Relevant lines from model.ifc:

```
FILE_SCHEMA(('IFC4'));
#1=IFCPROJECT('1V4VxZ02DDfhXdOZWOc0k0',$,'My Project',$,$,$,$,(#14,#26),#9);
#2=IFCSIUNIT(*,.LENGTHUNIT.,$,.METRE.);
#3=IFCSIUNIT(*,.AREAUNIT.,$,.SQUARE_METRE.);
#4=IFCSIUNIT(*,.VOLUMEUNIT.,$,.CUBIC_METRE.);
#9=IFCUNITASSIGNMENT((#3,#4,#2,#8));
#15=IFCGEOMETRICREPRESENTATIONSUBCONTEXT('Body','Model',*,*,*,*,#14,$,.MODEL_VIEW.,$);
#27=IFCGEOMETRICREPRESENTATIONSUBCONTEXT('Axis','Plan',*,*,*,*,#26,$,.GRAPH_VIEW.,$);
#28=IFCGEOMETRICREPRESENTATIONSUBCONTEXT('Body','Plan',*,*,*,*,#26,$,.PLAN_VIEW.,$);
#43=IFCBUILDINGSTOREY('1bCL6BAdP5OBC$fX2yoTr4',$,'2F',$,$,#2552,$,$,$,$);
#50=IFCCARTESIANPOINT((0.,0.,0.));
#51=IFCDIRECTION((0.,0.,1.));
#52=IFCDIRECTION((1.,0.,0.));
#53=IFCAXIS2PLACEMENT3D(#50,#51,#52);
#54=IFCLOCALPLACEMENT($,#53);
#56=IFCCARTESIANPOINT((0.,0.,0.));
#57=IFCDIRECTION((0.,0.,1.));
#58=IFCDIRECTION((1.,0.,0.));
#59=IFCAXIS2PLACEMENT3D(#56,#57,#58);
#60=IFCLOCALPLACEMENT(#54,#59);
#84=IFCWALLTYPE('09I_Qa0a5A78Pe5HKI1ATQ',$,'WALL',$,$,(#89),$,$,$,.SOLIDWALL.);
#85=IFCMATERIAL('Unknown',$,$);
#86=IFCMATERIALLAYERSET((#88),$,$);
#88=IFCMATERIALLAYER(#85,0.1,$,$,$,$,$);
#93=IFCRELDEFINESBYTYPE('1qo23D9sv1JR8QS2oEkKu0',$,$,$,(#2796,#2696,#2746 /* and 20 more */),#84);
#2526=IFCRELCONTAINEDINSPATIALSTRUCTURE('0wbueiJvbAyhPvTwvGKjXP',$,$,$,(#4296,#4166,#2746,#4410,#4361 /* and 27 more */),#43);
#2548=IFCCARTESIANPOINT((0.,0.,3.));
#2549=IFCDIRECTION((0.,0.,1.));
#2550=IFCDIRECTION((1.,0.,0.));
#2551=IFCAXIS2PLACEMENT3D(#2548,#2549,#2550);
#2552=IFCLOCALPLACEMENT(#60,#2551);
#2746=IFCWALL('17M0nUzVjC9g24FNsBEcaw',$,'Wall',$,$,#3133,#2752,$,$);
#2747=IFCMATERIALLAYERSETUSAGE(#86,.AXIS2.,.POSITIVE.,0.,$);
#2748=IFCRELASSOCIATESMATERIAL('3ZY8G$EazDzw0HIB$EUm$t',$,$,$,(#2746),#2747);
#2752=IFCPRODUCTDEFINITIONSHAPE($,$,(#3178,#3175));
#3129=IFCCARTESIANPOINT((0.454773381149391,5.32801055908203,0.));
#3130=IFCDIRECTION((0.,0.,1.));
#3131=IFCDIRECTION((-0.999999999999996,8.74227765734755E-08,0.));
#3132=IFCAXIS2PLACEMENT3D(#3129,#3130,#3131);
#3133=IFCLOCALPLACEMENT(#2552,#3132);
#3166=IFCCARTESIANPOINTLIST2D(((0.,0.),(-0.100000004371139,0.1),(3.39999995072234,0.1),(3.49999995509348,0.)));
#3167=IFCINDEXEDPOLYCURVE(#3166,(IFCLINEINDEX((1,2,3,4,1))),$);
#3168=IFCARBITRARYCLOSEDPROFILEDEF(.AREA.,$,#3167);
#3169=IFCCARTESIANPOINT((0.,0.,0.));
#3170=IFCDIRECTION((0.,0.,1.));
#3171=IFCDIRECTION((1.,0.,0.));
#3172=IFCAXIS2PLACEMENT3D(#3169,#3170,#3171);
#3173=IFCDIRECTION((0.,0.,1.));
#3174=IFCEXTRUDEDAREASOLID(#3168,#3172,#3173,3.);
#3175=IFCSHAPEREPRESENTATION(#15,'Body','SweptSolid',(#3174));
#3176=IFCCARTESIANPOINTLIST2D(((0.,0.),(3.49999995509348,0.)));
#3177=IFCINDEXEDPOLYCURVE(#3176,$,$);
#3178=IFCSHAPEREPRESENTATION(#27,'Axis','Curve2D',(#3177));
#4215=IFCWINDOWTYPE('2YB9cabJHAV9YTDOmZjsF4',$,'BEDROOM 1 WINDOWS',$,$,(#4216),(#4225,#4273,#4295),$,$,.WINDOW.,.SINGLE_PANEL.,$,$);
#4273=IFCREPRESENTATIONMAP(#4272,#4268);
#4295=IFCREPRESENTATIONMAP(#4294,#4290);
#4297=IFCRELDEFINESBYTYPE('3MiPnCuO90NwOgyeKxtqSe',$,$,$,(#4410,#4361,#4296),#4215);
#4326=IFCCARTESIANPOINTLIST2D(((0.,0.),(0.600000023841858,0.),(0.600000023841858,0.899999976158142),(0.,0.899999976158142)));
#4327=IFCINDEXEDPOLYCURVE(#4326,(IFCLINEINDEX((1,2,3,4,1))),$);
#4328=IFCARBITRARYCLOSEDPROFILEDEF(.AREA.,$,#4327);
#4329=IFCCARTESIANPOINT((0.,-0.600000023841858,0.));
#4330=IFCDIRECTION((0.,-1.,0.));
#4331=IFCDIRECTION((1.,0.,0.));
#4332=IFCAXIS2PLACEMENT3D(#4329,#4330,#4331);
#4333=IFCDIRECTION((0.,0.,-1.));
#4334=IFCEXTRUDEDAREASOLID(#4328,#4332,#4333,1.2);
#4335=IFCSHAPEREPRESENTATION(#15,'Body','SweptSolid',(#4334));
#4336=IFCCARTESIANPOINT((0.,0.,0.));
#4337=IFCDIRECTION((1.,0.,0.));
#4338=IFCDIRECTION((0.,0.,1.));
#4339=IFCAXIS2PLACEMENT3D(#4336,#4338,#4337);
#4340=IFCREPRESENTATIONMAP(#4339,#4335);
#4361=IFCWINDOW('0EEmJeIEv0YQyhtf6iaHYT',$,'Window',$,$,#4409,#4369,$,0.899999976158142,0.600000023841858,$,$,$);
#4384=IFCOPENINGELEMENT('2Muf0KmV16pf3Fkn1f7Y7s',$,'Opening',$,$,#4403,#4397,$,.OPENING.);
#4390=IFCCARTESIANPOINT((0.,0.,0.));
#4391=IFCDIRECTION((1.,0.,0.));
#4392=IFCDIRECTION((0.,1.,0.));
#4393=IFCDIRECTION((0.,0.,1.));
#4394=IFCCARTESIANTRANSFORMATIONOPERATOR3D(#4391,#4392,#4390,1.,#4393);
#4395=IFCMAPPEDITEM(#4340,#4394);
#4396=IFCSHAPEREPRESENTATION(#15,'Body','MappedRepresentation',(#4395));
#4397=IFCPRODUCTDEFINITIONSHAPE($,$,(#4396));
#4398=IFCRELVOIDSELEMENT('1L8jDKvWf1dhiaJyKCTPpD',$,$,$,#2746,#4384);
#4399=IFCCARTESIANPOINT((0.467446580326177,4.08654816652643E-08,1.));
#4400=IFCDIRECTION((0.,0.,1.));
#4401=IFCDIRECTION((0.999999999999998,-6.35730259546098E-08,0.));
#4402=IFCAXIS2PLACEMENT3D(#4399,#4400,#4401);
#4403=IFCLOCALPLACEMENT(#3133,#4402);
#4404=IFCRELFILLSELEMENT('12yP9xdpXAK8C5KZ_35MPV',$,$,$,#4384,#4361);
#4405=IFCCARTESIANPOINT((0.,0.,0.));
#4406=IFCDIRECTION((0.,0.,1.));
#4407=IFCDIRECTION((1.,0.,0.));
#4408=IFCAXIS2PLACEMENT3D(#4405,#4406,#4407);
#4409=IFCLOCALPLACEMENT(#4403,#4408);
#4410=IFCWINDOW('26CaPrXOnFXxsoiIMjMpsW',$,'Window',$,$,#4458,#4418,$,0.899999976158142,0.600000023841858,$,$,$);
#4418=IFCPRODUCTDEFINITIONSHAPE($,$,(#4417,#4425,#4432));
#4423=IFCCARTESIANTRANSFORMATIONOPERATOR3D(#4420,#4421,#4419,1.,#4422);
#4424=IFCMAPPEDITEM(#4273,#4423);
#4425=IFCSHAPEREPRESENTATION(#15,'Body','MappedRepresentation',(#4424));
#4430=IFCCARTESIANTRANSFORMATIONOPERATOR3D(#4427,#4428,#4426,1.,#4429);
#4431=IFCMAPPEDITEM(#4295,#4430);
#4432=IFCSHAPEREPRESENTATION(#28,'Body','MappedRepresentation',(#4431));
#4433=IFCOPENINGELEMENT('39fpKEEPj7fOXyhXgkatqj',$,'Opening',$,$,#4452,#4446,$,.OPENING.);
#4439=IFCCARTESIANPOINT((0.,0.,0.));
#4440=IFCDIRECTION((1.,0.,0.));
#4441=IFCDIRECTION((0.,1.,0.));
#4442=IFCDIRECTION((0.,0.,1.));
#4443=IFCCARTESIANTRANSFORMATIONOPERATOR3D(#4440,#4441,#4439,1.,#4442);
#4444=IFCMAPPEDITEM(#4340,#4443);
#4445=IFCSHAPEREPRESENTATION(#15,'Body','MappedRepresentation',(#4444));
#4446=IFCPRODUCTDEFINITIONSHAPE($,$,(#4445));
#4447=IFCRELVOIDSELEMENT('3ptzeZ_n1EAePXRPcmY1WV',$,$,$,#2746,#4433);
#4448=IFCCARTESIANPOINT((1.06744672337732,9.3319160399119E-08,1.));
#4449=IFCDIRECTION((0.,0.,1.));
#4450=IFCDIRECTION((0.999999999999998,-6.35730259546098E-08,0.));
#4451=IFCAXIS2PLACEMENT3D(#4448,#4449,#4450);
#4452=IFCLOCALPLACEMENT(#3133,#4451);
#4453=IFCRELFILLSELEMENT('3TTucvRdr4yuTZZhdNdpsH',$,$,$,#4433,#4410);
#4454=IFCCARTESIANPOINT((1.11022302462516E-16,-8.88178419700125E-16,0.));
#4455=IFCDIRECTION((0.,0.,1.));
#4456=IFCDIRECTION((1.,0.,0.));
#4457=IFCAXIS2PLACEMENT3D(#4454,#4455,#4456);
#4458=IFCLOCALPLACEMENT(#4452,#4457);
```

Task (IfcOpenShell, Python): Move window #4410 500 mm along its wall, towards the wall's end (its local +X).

```python
import ifcopenshell
import ifcopenshell.api.geometry
import ifcopenshell.util.placement

model = ifcopenshell.open("model.ifc")

window = model.by_guid("26CaPrXOnFXxsoiIMjMpsW")
opening = window.FillsVoids[0].RelatingOpeningElement
wall = opening.VoidsElements[0].RelatingBuildingElement

wall_matrix = ifcopenshell.util.placement.get_local_placement(wall.ObjectPlacement)
shift = wall_matrix[:3, 0] * 0.5
before = ifcopenshell.util.placement.get_local_placement(window.ObjectPlacement)[:3, 3].copy()

# The window is placed relative to its opening, so it follows when the opening moves.
matrix = ifcopenshell.util.placement.get_local_placement(opening.ObjectPlacement)
matrix[:3, 3] += shift
ifcopenshell.api.geometry.edit_object_placement(
    model, product=opening, matrix=matrix, is_si=False, should_transform_children=True
)

after = ifcopenshell.util.placement.get_local_placement(window.ObjectPlacement)[:3, 3]
print("window moved by", (after - before).round(3) + 0.0)

model.write("model-out.ifc")
```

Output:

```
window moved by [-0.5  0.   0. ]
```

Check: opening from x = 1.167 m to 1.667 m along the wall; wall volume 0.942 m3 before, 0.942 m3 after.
